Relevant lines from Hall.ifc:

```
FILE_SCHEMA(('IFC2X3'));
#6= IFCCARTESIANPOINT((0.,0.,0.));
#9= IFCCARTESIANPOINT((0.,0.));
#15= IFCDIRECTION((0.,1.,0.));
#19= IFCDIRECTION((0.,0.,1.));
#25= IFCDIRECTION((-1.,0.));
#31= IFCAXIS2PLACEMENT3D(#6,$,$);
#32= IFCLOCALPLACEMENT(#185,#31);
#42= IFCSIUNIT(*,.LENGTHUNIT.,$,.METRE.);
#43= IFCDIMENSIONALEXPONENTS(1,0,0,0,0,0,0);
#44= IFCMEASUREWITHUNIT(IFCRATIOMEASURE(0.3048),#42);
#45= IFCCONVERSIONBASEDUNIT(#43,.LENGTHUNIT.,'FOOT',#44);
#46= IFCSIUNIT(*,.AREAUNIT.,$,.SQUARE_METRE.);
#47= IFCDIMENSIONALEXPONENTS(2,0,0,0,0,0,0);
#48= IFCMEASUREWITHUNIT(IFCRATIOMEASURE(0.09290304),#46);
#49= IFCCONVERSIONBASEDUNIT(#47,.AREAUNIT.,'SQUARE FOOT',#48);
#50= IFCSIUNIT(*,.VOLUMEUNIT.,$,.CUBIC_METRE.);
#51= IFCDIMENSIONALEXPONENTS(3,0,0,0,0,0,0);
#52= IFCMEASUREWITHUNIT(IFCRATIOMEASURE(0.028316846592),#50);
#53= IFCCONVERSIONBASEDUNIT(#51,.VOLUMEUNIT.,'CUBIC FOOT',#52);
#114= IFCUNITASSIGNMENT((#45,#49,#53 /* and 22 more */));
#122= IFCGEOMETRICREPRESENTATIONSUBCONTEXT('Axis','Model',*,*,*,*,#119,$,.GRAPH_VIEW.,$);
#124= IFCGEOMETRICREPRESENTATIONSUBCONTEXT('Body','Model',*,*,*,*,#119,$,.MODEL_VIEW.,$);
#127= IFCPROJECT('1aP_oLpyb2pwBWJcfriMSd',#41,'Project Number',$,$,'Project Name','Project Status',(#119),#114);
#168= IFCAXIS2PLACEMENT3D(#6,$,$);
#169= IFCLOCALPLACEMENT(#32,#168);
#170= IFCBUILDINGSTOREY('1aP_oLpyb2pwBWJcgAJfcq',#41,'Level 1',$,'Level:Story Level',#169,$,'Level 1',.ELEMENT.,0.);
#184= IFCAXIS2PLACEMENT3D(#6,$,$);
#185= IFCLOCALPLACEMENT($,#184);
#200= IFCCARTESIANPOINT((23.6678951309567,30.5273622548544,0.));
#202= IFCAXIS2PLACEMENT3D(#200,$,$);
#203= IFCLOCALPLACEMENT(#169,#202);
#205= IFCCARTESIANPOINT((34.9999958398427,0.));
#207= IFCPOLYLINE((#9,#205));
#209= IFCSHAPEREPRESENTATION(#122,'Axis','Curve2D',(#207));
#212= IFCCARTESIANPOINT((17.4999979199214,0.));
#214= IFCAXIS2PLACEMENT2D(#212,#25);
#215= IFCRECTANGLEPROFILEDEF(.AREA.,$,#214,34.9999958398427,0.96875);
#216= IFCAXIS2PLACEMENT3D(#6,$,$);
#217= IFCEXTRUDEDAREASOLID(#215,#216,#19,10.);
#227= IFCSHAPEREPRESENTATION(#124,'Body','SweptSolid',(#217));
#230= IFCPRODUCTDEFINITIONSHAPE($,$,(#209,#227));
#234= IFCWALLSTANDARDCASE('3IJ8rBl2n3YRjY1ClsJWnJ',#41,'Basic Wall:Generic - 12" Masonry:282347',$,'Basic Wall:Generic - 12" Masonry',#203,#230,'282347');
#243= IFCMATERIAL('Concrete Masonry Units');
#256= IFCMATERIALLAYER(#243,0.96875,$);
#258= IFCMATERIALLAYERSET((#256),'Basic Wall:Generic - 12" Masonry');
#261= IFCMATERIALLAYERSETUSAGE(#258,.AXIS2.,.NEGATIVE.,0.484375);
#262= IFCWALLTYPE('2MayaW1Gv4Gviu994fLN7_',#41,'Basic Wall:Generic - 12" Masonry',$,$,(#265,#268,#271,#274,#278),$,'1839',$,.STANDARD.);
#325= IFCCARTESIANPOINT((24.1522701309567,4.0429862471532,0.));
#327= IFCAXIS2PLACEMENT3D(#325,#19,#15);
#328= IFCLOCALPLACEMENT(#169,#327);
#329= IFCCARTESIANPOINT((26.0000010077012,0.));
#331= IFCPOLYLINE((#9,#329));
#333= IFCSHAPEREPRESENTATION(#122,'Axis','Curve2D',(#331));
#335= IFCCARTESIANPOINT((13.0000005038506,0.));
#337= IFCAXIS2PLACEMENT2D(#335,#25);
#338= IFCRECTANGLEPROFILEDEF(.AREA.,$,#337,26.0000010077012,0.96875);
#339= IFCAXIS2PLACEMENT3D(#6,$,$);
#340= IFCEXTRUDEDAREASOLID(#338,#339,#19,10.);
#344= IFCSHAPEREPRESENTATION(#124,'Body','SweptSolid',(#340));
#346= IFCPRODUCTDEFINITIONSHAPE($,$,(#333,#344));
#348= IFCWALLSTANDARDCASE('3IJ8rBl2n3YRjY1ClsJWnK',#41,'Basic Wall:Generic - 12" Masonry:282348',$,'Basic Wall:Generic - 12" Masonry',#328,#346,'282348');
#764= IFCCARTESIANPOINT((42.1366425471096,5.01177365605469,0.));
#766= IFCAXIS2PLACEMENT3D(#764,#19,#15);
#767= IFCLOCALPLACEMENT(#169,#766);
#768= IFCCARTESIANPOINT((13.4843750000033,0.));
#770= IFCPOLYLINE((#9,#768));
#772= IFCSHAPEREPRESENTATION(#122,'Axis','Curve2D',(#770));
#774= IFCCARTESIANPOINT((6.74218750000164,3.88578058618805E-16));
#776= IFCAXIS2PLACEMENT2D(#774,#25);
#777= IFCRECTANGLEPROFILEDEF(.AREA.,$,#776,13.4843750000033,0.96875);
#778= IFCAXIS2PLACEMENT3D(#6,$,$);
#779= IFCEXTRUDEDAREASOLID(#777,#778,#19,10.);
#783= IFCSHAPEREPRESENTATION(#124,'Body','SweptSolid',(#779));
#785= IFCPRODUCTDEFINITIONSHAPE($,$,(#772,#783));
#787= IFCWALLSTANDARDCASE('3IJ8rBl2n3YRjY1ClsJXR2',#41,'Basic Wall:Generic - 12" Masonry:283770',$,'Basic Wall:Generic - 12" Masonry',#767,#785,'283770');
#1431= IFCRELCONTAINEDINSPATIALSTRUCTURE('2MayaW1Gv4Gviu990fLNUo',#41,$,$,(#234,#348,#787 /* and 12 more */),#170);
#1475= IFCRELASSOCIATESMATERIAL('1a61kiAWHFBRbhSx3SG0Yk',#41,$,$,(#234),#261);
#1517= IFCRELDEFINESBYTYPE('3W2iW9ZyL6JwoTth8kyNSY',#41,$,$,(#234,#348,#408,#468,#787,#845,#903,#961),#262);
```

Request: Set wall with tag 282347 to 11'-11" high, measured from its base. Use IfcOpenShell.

```python
import ifcopenshell
import ifcopenshell.geom
import ifcopenshell.util.representation
import ifcopenshell.util.shape
import ifcopenshell.util.unit

model = ifcopenshell.open("Hall.ifc")
unit_scale = ifcopenshell.util.unit.calculate_unit_scale(model)
settings = ifcopenshell.geom.settings()


def volume(element):
    """Net volume in cubic metres, openings subtracted."""
    shape = ifcopenshell.geom.create_shape(settings, element)
    return ifcopenshell.util.shape.get_volume(shape.geometry)


wall = model.by_id(234)
before = volume(wall)

body = ifcopenshell.util.representation.get_representation(wall, "Model", "Body")
solid = body.Items[0]
old_height = solid.Depth
solid.Depth = 143 * 0.0254 / unit_scale
after = volume(wall)

print(f"height {old_height:g} -> {solid.Depth:g}, volume {before:.3f} -> {after:.3f} m3")

model.write("Hall_rev.ifc")
```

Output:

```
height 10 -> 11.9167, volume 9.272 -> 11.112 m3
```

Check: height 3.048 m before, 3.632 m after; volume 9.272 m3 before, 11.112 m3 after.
